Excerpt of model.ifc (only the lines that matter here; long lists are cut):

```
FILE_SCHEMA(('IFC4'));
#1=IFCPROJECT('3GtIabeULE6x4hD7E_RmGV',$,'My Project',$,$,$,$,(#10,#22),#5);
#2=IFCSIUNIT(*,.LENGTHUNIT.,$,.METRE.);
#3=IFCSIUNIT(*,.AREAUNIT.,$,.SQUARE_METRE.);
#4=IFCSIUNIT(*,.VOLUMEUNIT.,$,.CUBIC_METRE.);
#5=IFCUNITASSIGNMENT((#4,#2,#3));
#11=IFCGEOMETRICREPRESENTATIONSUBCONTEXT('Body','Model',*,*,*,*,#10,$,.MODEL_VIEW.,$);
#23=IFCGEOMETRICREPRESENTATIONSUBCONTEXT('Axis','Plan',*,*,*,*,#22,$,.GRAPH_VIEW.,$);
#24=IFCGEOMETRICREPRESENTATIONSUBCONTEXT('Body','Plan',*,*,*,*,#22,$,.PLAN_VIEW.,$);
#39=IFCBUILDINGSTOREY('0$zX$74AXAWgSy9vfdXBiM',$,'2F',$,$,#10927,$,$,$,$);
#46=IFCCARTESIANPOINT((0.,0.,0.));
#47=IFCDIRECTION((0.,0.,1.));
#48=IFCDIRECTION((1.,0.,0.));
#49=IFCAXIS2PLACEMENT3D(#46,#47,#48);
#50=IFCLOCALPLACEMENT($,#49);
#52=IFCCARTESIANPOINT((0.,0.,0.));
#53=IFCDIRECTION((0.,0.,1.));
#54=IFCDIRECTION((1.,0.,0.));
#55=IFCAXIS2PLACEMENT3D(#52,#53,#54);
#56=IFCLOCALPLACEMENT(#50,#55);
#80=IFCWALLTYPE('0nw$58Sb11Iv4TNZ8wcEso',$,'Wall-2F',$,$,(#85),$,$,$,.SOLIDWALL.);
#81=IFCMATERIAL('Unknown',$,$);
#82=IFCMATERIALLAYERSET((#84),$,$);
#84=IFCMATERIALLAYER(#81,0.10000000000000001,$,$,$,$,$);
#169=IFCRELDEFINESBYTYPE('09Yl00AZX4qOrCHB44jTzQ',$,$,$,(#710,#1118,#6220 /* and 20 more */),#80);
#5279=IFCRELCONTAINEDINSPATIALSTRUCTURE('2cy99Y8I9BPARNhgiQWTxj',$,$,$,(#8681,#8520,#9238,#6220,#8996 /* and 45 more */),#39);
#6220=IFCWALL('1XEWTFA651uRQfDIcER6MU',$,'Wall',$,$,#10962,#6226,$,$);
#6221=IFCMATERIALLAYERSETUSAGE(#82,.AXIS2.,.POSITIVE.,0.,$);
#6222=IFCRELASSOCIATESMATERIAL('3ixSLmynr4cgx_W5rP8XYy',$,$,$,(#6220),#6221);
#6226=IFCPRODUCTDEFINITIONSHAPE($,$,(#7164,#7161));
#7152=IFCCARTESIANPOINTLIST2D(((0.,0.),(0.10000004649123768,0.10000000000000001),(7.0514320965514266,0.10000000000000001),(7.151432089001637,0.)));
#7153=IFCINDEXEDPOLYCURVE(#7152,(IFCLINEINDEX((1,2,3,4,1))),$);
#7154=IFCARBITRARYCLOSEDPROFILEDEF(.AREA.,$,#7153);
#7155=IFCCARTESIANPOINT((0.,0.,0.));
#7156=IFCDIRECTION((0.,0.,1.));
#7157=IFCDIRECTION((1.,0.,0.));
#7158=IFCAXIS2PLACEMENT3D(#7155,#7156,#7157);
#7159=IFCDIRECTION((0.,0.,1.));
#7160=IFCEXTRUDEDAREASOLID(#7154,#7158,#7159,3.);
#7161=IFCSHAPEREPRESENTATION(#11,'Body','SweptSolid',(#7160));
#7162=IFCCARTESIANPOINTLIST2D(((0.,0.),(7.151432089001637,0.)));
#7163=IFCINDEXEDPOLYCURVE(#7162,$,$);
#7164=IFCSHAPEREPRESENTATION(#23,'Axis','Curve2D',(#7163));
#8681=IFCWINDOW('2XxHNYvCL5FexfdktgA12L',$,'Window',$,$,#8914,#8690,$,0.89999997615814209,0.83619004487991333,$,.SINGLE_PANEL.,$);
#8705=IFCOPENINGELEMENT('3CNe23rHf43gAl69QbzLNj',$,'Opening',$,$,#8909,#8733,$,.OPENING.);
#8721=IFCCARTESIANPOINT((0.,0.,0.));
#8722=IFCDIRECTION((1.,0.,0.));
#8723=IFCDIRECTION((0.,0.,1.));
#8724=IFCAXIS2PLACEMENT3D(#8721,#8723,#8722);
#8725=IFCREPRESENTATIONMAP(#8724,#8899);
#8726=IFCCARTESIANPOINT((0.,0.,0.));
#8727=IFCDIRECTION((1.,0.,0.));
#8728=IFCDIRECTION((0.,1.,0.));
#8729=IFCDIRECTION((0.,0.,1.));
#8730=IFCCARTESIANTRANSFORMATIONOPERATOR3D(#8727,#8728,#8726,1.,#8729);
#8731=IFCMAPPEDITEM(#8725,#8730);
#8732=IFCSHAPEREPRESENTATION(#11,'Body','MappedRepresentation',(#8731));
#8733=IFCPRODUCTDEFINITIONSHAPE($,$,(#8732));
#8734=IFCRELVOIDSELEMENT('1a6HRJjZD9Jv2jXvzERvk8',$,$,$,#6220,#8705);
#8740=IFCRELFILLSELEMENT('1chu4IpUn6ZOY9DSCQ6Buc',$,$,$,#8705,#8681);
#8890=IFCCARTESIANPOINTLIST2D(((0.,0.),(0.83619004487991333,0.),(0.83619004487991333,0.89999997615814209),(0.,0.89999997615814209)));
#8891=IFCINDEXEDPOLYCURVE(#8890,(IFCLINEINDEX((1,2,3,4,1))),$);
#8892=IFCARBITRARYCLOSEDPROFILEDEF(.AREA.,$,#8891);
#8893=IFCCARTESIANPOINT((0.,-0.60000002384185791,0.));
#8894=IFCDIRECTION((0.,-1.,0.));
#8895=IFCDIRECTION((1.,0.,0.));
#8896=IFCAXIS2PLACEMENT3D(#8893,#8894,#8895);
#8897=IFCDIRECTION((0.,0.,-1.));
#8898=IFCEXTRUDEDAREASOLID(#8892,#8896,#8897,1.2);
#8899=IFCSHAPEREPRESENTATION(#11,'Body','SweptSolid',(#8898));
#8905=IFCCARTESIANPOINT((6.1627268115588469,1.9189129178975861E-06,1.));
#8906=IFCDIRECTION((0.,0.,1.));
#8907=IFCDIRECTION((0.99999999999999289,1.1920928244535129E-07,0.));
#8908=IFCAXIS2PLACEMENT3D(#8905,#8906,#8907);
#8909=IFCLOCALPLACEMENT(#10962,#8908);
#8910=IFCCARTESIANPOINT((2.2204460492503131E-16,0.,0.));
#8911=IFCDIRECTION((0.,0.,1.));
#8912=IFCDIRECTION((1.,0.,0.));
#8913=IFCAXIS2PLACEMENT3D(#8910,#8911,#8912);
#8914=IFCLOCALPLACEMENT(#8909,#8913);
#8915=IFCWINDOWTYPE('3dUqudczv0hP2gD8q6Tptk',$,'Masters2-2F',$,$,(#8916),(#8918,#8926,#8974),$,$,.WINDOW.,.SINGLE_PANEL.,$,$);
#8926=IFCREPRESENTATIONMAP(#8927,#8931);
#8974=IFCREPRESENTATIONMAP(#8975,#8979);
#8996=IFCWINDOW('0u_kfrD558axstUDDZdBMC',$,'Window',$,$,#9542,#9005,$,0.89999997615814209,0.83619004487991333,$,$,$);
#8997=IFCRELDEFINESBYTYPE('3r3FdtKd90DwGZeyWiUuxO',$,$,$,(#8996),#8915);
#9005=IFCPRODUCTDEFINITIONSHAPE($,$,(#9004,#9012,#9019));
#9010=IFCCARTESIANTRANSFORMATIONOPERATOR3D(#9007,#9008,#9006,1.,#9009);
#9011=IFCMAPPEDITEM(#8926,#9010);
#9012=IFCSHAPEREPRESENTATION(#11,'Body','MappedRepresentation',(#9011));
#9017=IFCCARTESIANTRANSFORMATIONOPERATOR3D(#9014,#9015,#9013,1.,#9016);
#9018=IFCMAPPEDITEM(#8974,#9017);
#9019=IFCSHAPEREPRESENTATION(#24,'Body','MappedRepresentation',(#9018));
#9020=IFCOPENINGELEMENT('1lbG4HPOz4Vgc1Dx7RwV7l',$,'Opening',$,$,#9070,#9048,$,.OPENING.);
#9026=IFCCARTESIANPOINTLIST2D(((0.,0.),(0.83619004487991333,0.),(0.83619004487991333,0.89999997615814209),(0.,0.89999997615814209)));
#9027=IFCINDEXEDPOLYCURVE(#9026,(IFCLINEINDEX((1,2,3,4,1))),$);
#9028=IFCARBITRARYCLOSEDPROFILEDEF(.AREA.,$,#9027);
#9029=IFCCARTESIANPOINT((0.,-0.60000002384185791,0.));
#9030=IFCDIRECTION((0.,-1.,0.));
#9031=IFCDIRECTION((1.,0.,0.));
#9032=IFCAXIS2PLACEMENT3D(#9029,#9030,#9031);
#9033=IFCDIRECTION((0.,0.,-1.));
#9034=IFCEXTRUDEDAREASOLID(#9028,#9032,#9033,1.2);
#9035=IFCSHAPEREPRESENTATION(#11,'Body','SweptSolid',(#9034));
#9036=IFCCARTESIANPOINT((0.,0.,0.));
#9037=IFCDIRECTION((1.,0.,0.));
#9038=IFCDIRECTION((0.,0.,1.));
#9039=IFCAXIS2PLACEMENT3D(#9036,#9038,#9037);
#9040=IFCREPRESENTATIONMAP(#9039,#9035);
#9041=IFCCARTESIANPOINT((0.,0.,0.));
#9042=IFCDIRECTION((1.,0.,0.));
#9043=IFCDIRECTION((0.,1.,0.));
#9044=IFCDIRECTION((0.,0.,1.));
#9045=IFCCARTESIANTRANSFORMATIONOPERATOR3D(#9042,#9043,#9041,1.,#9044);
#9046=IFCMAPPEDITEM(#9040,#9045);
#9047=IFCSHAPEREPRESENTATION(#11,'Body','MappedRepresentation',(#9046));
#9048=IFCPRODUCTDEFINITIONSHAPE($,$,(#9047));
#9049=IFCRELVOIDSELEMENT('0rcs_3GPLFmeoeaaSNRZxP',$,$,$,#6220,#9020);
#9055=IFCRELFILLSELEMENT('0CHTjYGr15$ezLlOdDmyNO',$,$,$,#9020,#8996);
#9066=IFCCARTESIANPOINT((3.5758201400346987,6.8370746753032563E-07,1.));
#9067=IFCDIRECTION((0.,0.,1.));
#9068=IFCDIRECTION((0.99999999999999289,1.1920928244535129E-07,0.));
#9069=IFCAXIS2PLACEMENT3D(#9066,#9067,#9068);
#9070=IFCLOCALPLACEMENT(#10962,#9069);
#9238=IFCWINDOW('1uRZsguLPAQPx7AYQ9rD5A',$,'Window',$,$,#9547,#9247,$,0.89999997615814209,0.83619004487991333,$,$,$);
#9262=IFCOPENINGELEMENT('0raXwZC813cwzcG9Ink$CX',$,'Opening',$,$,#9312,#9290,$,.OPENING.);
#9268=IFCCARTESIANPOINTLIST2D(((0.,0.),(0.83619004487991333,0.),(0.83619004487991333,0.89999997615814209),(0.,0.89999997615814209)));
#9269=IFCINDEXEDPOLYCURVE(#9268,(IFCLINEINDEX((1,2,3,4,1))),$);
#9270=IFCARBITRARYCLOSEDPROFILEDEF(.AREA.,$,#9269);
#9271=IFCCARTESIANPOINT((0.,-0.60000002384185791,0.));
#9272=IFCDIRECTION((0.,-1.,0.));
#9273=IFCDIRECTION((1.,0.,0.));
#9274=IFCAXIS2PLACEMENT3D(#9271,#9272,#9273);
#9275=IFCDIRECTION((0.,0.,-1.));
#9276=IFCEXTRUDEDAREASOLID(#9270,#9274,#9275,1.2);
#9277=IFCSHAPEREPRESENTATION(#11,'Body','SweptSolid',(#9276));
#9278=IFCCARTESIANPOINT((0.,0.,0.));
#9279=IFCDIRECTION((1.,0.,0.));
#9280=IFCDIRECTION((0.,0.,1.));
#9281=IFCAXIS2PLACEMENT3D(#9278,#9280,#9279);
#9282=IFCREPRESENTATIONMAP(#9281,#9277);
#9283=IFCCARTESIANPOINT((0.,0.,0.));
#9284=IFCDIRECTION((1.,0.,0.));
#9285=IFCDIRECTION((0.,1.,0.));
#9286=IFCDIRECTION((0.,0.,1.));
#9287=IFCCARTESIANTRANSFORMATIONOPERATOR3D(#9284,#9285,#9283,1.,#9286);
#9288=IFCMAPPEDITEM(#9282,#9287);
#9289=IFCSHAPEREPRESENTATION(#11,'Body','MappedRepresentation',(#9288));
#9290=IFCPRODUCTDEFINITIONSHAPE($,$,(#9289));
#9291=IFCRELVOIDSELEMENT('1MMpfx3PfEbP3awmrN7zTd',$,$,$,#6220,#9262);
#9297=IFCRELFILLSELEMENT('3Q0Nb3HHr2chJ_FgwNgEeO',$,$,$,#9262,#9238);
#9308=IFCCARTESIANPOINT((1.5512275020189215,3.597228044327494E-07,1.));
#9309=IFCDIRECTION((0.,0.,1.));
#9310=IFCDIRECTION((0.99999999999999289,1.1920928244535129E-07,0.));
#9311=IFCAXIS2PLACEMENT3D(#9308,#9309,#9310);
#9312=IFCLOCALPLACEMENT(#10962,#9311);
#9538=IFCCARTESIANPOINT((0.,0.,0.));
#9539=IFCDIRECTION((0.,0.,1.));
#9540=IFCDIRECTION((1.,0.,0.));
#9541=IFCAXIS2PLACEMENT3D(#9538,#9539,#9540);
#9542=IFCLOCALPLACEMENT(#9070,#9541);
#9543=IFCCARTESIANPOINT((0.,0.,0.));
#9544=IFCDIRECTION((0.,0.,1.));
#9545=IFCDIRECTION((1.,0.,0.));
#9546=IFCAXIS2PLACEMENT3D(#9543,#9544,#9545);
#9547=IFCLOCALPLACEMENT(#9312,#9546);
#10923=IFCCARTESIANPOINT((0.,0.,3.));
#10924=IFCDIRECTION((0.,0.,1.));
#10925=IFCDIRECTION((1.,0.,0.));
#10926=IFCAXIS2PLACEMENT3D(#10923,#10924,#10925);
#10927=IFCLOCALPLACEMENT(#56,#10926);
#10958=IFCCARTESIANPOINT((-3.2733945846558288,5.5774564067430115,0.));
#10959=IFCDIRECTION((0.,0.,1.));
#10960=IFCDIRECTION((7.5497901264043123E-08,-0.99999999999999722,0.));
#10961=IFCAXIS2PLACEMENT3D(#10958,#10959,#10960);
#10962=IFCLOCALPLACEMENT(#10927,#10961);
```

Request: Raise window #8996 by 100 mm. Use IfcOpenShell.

```python
import numpy as np
import ifcopenshell
import ifcopenshell.api.geometry
import ifcopenshell.util.placement
import ifcopenshell.util.unit

model = ifcopenshell.open("model.ifc")
unit_scale = ifcopenshell.util.unit.calculate_unit_scale(model)

window = model.by_id(8996)
opening = window.FillsVoids[0].RelatingOpeningElement
dz = 0.1 / unit_scale

shift = np.array([0.0, 0.0, dz])
# The window is placed relative to its opening, so it follows when the opening moves.
matrix = ifcopenshell.util.placement.get_local_placement(opening.ObjectPlacement)
matrix[:3, 3] += shift
ifcopenshell.api.geometry.edit_object_placement(
    model, product=opening, matrix=matrix, is_si=False, should_transform_children=True
)

print(f"moved by {dz * unit_scale:+.3f} m")

model.write("model_updated.ifc")
```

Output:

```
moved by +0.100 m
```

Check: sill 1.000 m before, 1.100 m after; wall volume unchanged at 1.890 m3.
